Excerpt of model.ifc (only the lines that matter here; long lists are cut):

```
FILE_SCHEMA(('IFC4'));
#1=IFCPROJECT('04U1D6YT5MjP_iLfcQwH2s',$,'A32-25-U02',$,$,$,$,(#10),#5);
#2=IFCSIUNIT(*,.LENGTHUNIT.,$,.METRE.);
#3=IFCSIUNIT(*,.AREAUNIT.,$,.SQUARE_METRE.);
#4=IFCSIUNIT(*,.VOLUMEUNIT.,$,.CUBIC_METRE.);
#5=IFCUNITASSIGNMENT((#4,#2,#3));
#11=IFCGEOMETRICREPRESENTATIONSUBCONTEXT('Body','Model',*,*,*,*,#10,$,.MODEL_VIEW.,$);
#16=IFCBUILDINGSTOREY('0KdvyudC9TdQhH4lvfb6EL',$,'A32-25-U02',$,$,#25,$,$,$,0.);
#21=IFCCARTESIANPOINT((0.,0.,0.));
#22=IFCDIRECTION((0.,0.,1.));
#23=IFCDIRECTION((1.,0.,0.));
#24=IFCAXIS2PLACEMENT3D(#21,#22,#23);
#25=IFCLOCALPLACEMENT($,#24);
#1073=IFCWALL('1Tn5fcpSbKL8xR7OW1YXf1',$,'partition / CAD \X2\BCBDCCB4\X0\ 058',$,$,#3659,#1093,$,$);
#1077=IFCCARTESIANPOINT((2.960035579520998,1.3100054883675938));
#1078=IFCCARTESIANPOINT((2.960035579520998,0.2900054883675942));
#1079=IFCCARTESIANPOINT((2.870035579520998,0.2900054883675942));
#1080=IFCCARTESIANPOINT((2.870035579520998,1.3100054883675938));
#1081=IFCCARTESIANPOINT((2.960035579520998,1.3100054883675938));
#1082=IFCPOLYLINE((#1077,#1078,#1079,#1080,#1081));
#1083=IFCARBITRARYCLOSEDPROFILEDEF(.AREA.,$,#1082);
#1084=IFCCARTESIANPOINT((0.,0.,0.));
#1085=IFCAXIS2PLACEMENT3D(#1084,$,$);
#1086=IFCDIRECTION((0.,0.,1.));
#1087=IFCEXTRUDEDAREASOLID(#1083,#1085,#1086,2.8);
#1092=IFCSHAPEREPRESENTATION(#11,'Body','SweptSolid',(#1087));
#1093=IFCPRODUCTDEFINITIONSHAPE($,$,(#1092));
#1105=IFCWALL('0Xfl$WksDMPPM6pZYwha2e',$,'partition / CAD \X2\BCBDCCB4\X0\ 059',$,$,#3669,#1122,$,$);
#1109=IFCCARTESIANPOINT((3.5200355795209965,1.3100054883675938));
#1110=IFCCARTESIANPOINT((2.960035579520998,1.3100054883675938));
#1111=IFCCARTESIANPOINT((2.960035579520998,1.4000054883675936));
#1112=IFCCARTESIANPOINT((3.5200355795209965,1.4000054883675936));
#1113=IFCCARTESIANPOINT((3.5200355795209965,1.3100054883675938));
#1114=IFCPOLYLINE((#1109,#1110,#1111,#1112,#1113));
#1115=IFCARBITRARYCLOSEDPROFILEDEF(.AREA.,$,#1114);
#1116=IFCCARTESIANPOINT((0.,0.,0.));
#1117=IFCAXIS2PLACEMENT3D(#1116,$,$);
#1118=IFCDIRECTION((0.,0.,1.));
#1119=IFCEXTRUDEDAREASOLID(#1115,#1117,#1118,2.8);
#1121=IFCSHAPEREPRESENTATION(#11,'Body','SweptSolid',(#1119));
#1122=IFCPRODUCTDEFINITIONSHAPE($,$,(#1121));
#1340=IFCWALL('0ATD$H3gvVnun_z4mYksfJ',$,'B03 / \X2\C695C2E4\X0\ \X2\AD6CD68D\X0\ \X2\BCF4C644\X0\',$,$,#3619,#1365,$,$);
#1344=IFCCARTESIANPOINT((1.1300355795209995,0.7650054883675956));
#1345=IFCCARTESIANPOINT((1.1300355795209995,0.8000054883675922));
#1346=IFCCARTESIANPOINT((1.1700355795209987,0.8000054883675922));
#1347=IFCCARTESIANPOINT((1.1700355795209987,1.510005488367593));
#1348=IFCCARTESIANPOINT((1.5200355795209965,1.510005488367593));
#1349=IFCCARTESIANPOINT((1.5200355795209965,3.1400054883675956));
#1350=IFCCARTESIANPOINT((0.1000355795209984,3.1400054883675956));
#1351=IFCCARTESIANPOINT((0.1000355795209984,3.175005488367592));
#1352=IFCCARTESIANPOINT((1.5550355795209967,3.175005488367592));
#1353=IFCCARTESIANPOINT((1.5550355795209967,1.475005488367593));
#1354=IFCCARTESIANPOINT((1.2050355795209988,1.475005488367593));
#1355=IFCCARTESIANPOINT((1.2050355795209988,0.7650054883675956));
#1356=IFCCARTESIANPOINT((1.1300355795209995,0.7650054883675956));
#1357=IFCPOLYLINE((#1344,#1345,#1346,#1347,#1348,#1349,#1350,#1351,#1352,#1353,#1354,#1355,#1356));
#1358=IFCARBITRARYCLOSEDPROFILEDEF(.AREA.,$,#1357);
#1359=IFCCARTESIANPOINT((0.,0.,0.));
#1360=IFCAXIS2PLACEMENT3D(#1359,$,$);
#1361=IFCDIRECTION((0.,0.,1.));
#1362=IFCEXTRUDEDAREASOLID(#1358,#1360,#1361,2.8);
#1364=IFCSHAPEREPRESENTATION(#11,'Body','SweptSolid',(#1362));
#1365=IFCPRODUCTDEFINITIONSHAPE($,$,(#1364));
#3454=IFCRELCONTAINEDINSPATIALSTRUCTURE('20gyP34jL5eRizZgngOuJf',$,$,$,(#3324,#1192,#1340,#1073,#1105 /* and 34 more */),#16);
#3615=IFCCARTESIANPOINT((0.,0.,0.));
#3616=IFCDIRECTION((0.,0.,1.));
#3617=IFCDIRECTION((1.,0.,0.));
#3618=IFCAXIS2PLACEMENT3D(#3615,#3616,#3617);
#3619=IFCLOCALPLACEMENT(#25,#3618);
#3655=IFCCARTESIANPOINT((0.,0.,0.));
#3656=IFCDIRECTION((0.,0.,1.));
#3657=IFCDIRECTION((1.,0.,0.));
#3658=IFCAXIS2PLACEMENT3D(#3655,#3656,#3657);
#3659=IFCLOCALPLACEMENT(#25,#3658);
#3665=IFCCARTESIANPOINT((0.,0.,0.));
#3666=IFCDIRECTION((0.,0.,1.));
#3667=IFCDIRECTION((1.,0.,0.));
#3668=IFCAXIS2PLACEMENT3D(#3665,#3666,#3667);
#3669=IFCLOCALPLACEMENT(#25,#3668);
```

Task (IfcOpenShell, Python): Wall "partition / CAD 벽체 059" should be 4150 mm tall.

```python
import ifcopenshell
import ifcopenshell.geom
import ifcopenshell.util.representation
import ifcopenshell.util.shape

model = ifcopenshell.open("model.ifc")
settings = ifcopenshell.geom.settings()


def volume(element):
    """Net volume in cubic metres, openings subtracted."""
    shape = ifcopenshell.geom.create_shape(settings, element)
    return ifcopenshell.util.shape.get_volume(shape.geometry)


wall = model.by_guid("0Xfl$WksDMPPM6pZYwha2e")
before = volume(wall)

body = ifcopenshell.util.representation.get_representation(wall, "Model", "Body")
solid = body.Items[0]
old_height = solid.Depth
solid.Depth = 4.15
after = volume(wall)

print(f"height {old_height:g} -> {solid.Depth:g}, volume {before:.3f} -> {after:.3f} m3")

model.write("model_v2.ifc")
```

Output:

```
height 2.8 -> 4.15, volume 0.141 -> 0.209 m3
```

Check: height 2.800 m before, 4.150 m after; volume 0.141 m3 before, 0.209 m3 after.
